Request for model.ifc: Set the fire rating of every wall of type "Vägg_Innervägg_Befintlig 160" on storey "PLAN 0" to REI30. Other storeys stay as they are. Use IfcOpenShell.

First a look at what the model holds.

```python
import ifcopenshell
import ifcopenshell.util.element

model = ifcopenshell.open("model.ifc")
print(model.schema)
storey = next(s for s in model.by_type("IfcBuildingStorey") if s.Name == "PLAN 0")
walls = [e for e in ifcopenshell.util.element.get_decomposition(storey) if e.is_a("IfcWall")]
seen = {}
for e in walls:
    element_type = ifcopenshell.util.element.get_type(e)
    key = (element_type.Name if element_type != e and element_type else None, ifcopenshell.util.element.get_pset(e, "Pset_WallCommon", "FireRating"))
    seen[key] = seen.get(key, 0) + 1
for (name, value), count in sorted(seen.items(), key=str):
    print(count, "x", name, "|", value)
```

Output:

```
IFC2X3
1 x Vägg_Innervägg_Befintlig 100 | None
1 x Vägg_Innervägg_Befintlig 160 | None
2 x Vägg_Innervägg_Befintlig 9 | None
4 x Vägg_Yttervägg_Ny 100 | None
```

```python
import ifcopenshell
import ifcopenshell.api.pset
import ifcopenshell.util.element

model = ifcopenshell.open("model.ifc")

storey = next(s for s in model.by_type("IfcBuildingStorey") if s.Name == "PLAN 0")
walls = [e for e in ifcopenshell.util.element.get_decomposition(storey) if e.is_a("IfcWall")]

count = 0
for e in walls:
    element_type = ifcopenshell.util.element.get_type(e)
    if element_type in (None, e) or element_type.Name != "Vägg_Innervägg_Befintlig 160":
        continue
    # add_pset returns the element's existing set when there is one.
    pset = ifcopenshell.api.pset.add_pset(model, product=e, name="Pset_WallCommon")
    ifcopenshell.api.pset.edit_pset(model, pset=pset, properties={"FireRating": "REI30"})
    count += 1

print(count, "walls updated")

model.write("model-out.ifc")
```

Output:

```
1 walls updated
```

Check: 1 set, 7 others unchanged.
